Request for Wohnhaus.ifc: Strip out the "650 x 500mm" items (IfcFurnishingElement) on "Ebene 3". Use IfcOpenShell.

First a look at what the model holds.

```python
import ifcopenshell
import ifcopenshell.util.element

model = ifcopenshell.open("Wohnhaus.ifc")
print(model.schema)
storey = next(s for s in model.by_type("IfcBuildingStorey") if s.Name == "Ebene 3")
furniture = [e for e in ifcopenshell.util.element.get_decomposition(storey) if e.is_a("IfcFurnishingElement")]
seen = {}
for e in furniture:
    element_type = ifcopenshell.util.element.get_type(e)
    name = element_type.Name if element_type not in (None, e) else None
    seen[name] = seen.get(name, 0) + 1
for name, count in sorted(seen.items(), key=str):
    print(count, "x", name)
```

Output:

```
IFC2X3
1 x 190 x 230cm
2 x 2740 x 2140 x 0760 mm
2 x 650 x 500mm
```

```python
import ifcopenshell
import ifcopenshell.api.root
import ifcopenshell.util.element

model = ifcopenshell.open("Wohnhaus.ifc")

storey = next(s for s in model.by_type("IfcBuildingStorey") if s.Name == "Ebene 3")
furniture = [e for e in ifcopenshell.util.element.get_decomposition(storey) if e.is_a("IfcFurnishingElement")]
targets = [e for e in furniture if (t := ifcopenshell.util.element.get_type(e)) not in (None, e) and t.Name == "650 x 500mm"]

for e in targets:
    ifcopenshell.api.root.remove_product(model, product=e)
print(len(targets), "removed")

model.write("Wohnhaus_edited.ifc")
```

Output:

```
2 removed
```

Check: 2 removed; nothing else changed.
